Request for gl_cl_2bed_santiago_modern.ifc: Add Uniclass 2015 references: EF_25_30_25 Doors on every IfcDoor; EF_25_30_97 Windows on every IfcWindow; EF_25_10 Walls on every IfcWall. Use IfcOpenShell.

First a look at what the model holds.

```python
import ifcopenshell

model = ifcopenshell.open("gl_cl_2bed_santiago_modern.ifc")
print(model.schema)
print("classifications:", [c.Name for c in model.by_type("IfcClassification")])
for ifc_class in ("IfcDoor", "IfcRoof", "IfcStair", "IfcWall", "IfcWindow"):
    print(ifc_class, len(model.by_type(ifc_class)))
```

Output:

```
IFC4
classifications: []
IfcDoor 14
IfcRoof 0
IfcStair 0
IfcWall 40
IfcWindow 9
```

```python
import ifcopenshell
import ifcopenshell.api.classification

model = ifcopenshell.open("gl_cl_2bed_santiago_modern.ifc")

system = ifcopenshell.api.classification.add_classification(model, classification="Uniclass 2015")

codes = {
    "IfcDoor": ("EF_25_30_25", "Doors"),
    "IfcWindow": ("EF_25_30_97", "Windows"),
    "IfcWall": ("EF_25_10", "Walls"),
}
for ifc_class, (code, name) in codes.items():
    products = model.by_type(ifc_class)
    ifcopenshell.api.classification.add_reference(
        model, products=products, classification=system, identification=code, name=name
    )
    print(code, len(products))

model.write("gl_cl_2bed_santiago_modern_edited.ifc")
```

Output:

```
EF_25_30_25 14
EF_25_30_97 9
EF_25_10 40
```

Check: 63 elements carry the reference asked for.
